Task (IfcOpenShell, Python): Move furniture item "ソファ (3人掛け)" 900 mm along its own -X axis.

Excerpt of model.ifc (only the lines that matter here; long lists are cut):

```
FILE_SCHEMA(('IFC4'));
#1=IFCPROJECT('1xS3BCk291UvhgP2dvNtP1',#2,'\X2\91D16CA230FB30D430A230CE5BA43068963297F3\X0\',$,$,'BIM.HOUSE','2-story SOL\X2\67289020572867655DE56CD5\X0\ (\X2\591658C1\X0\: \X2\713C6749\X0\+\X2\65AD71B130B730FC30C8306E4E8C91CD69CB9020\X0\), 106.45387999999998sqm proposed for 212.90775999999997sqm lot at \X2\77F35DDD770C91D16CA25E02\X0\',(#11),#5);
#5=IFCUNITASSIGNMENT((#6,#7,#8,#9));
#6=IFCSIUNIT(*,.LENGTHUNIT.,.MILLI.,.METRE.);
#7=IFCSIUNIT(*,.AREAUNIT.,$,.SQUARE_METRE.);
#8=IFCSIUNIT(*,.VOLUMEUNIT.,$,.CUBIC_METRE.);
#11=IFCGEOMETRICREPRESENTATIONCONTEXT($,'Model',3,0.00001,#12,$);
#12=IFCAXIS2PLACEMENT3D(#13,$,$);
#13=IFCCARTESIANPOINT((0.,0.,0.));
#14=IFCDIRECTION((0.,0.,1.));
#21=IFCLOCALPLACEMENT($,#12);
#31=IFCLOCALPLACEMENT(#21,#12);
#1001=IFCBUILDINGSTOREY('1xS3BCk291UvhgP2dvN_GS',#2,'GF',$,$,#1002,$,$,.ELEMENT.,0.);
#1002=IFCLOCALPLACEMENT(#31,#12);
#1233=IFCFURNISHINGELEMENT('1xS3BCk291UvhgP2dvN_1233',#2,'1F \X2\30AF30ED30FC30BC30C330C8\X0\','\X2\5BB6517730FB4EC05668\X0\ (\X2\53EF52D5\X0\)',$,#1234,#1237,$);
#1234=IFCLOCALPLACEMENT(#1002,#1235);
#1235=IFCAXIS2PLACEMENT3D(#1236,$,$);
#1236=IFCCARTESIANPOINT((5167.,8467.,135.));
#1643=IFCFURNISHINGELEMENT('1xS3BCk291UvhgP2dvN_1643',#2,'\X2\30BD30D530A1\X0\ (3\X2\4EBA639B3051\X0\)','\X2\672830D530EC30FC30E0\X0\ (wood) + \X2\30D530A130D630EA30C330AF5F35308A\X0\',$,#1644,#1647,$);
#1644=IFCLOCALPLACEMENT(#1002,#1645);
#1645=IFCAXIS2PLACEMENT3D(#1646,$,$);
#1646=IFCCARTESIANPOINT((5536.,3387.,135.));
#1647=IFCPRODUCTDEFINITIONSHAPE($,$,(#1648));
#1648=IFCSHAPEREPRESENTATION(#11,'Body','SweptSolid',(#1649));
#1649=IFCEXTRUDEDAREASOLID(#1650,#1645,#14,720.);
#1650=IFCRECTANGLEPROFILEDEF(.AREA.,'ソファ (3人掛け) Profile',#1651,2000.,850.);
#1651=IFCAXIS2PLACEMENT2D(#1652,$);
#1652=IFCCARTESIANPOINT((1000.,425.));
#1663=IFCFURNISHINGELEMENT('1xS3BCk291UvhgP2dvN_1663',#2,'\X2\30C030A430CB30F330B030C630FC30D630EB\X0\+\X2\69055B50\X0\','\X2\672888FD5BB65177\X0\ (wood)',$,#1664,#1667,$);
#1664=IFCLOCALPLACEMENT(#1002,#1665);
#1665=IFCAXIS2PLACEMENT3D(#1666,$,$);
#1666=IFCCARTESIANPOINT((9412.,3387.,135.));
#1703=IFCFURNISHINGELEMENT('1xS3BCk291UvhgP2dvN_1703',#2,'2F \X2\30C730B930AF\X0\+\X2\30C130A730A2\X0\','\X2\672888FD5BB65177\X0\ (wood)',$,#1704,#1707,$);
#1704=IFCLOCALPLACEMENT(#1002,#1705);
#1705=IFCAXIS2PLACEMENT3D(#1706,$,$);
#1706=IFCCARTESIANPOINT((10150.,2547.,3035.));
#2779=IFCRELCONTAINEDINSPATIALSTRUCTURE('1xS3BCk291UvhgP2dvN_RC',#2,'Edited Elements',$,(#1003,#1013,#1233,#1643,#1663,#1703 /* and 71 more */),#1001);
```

```python
import ifcopenshell
import ifcopenshell.api.geometry
import ifcopenshell.util.placement
import ifcopenshell.util.unit

model = ifcopenshell.open("model.ifc")
unit_scale = ifcopenshell.util.unit.calculate_unit_scale(model)

item = model.by_guid("1xS3BCk291UvhgP2dvN_1643")
matrix = ifcopenshell.util.placement.get_local_placement(item.ObjectPlacement)
matrix[:3, 3] -= matrix[:3, 0] * 0.9 / unit_scale
ifcopenshell.api.geometry.edit_object_placement(model, product=item, matrix=matrix, is_si=False)

print(ifcopenshell.util.placement.get_local_placement(item.ObjectPlacement).round(3) + 0.0)

model.write("model_updated.ifc")
```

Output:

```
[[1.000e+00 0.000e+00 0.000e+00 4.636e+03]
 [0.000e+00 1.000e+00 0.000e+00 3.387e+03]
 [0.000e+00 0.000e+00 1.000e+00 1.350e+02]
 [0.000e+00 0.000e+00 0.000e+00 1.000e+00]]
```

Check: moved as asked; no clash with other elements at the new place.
